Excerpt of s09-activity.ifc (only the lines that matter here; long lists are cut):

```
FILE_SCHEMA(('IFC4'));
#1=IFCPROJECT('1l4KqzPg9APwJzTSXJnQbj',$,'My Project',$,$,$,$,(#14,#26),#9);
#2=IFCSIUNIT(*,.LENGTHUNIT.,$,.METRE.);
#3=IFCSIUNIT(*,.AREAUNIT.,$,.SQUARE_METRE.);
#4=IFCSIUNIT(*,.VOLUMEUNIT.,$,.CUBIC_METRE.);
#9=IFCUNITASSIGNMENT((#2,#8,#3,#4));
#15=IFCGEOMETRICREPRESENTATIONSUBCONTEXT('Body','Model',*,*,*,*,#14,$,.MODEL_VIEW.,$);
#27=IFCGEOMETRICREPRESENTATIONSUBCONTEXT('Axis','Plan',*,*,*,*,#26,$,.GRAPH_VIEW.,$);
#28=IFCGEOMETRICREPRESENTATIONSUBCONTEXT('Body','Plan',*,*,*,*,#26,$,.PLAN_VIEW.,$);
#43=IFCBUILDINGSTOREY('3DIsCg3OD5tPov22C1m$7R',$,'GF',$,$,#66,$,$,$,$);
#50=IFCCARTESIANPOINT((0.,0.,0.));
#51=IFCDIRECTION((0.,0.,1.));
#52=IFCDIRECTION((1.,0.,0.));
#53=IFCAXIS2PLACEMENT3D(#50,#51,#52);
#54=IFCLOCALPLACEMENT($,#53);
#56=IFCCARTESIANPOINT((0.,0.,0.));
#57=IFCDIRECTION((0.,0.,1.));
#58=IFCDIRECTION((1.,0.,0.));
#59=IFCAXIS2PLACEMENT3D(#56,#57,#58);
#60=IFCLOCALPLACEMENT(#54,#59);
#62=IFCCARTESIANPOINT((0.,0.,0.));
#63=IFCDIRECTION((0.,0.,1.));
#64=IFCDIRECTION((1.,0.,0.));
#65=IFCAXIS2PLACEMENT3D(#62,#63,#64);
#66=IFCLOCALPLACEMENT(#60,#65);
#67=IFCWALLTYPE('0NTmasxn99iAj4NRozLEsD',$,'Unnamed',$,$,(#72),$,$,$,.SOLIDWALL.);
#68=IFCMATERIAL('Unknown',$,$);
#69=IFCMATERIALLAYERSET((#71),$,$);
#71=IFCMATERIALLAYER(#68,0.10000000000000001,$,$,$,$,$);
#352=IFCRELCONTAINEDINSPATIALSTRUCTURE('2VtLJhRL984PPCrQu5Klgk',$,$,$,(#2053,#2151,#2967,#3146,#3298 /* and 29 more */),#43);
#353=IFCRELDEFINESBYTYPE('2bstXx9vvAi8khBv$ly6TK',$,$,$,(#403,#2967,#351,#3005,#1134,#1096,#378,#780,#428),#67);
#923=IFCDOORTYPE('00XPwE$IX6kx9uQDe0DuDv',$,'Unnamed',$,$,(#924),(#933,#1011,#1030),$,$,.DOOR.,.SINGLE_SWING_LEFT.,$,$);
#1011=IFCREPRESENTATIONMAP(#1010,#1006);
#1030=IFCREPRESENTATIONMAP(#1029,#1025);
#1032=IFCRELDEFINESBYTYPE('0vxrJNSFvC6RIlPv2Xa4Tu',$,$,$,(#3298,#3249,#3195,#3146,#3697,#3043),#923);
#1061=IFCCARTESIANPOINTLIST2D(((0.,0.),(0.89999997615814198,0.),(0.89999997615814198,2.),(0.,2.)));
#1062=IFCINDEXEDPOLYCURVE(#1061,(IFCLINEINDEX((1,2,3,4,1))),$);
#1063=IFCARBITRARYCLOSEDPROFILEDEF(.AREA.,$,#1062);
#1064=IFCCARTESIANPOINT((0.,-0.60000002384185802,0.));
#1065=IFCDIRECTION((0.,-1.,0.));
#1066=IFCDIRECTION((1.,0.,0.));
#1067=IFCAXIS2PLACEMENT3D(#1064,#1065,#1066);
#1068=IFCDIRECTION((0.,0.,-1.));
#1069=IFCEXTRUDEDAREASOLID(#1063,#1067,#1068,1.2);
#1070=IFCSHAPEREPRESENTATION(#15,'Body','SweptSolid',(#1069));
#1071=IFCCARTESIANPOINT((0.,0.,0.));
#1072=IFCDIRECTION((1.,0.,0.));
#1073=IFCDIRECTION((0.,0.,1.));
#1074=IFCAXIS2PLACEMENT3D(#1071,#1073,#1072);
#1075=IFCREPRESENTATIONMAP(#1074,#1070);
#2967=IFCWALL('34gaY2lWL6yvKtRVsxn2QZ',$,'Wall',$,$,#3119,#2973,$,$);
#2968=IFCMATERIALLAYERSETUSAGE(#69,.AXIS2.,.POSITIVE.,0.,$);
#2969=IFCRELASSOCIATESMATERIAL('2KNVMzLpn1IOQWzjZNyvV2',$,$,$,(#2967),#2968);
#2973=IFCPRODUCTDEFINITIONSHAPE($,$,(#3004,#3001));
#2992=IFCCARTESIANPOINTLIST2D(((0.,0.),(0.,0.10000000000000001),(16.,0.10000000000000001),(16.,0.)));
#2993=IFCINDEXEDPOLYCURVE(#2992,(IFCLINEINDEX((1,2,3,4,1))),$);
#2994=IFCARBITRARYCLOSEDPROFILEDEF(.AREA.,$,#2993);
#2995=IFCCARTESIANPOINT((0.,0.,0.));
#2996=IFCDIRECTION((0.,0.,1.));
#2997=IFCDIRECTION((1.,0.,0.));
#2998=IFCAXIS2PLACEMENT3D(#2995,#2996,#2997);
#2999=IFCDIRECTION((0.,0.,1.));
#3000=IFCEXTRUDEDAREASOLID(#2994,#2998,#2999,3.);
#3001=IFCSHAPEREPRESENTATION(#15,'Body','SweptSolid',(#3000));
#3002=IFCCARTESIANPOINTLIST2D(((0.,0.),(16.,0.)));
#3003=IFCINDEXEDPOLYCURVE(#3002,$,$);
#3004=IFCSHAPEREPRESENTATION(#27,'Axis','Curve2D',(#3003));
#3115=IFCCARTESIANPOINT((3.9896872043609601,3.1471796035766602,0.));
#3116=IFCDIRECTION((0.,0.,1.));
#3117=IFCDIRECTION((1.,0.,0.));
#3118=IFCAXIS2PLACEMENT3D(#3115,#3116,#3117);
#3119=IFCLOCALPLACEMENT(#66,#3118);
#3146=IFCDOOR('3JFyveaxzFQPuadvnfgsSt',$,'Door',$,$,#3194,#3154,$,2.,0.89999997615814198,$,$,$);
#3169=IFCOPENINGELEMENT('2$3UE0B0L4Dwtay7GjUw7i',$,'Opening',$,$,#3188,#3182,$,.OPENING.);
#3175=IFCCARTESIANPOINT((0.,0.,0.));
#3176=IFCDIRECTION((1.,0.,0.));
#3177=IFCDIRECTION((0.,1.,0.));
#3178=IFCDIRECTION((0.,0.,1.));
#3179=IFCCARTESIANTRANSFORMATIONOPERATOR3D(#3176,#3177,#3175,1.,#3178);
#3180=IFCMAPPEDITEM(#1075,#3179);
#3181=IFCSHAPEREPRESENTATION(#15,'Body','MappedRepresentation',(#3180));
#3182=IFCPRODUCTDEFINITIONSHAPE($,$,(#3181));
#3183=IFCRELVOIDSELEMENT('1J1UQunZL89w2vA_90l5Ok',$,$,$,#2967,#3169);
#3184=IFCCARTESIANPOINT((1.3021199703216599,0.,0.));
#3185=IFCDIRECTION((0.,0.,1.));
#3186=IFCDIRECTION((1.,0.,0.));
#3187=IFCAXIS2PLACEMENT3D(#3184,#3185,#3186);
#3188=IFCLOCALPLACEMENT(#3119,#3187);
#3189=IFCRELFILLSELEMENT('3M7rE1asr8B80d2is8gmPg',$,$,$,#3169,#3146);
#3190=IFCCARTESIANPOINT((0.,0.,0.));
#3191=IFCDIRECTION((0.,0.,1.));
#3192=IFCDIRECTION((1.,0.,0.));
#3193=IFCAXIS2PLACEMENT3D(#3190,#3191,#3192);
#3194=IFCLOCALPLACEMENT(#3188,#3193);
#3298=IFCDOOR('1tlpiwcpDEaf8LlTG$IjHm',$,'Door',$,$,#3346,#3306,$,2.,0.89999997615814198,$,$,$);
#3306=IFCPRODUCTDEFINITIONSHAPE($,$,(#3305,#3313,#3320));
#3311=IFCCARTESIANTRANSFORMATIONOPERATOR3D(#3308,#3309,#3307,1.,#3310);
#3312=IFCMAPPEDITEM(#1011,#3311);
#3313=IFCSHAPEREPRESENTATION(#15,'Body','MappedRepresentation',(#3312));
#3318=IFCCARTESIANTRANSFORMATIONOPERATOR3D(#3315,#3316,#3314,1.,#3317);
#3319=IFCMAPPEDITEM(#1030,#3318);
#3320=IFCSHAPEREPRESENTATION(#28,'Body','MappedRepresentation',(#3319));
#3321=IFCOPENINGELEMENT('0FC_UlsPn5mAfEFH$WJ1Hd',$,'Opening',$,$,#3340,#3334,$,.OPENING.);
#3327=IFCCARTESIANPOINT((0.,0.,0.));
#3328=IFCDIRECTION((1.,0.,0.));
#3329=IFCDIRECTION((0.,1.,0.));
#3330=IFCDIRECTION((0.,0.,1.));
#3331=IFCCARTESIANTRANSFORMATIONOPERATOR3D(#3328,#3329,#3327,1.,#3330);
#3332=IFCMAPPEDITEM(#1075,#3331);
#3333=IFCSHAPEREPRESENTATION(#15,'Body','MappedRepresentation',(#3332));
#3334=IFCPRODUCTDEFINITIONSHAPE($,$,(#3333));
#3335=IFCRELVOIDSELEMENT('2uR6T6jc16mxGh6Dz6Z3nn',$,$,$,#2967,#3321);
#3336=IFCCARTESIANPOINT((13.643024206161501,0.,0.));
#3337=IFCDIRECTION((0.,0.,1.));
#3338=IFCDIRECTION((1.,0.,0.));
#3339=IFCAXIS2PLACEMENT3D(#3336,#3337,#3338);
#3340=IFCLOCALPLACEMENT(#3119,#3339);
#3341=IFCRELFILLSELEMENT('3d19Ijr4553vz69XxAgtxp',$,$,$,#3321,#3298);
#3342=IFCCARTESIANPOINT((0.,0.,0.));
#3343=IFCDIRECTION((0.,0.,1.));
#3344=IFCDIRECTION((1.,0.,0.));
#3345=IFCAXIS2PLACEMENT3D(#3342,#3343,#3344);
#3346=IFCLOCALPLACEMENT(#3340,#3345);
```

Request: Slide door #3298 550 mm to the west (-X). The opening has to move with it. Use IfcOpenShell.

```python
import ifcopenshell
import ifcopenshell.api.geometry
import ifcopenshell.util.placement
import ifcopenshell.util.unit

model = ifcopenshell.open("s09-activity.ifc")
unit_scale = ifcopenshell.util.unit.calculate_unit_scale(model)

door = model.by_id(3298)
opening = door.FillsVoids[0].RelatingOpeningElement
wall = opening.VoidsElements[0].RelatingBuildingElement

wall_matrix = ifcopenshell.util.placement.get_local_placement(wall.ObjectPlacement)
shift = wall_matrix[:3, 0] * -0.55 / unit_scale
before = ifcopenshell.util.placement.get_local_placement(door.ObjectPlacement)[:3, 3].copy()

# The door is placed relative to its opening, so it follows when the opening moves.
matrix = ifcopenshell.util.placement.get_local_placement(opening.ObjectPlacement)
matrix[:3, 3] += shift
ifcopenshell.api.geometry.edit_object_placement(
    model, product=opening, matrix=matrix, is_si=False, should_transform_children=True
)

after = ifcopenshell.util.placement.get_local_placement(door.ObjectPlacement)[:3, 3]
print("door moved by", (after - before).round(3) + 0.0)

model.write("s09-activity_updated.ifc")
```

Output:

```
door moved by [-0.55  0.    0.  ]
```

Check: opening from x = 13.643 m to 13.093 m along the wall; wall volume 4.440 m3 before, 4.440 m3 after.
